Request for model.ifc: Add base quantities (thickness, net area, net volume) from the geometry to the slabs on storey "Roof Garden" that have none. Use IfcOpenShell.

First a look at what the model holds.

```python
import ifcopenshell
import ifcopenshell.util.element
import ifcopenshell.util.unit

model = ifcopenshell.open("model.ifc")
print(model.schema)
for unit_type in ("LENGTHUNIT", "AREAUNIT", "VOLUMEUNIT"):
    print(unit_type, ifcopenshell.util.unit.calculate_unit_scale(model, unit_type))
storey = next(s for s in model.by_type("IfcBuildingStorey") if s.Name == "Roof Garden")
slabs = [e for e in ifcopenshell.util.element.get_decomposition(storey) if e.is_a("IfcSlab")]
for e in sorted(slabs, key=lambda e: e.id()):
    print(e.id(), e.is_a(), e.Name, list(ifcopenshell.util.element.get_psets(e, qtos_only=True)), sep=" | ")
```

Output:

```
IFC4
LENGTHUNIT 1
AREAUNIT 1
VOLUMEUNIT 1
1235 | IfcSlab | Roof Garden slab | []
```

```python
import ifcopenshell
import ifcopenshell.api.pset
import ifcopenshell.geom
import ifcopenshell.util.element
import ifcopenshell.util.shape
import ifcopenshell.util.unit

model = ifcopenshell.open("model.ifc")
unit_scale = ifcopenshell.util.unit.calculate_unit_scale(model)
area_scale = ifcopenshell.util.unit.calculate_unit_scale(model, "AREAUNIT")
volume_scale = ifcopenshell.util.unit.calculate_unit_scale(model, "VOLUMEUNIT")
settings = ifcopenshell.geom.settings()

storey = next(s for s in model.by_type("IfcBuildingStorey") if s.Name == "Roof Garden")
slabs = [e for e in ifcopenshell.util.element.get_decomposition(storey) if e.is_a("IfcSlab")]

for e in sorted(slabs, key=lambda e: e.id()):
    if ifcopenshell.util.element.get_psets(e, qtos_only=True, should_inherit=False):
        continue
    # Geometry comes back in metres, in the element's own axes.
    shape = ifcopenshell.geom.create_shape(settings, e)
    values = {
        "Width": ifcopenshell.util.shape.get_z(shape.geometry) / unit_scale,
        "NetArea": ifcopenshell.util.shape.get_footprint_area(shape.geometry) / area_scale,
        "NetVolume": ifcopenshell.util.shape.get_volume(shape.geometry) / volume_scale,
    }
    qto = ifcopenshell.api.pset.add_qto(model, product=e, name="Qto_SlabBaseQuantities")
    ifcopenshell.api.pset.edit_qto(model, qto=qto, properties=values)
    print(e.id(), {k: round(v, 3) for k, v in values.items()})

model.write("model_edited.ifc")
```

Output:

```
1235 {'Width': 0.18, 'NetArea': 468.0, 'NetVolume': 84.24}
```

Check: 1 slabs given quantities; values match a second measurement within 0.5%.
